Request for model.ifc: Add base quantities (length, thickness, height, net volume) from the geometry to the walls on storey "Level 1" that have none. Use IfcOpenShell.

First a look at what the model holds.

```python
import ifcopenshell
import ifcopenshell.util.element
import ifcopenshell.util.unit

model = ifcopenshell.open("model.ifc")
print(model.schema)
for unit_type in ("LENGTHUNIT", "AREAUNIT", "VOLUMEUNIT"):
    print(unit_type, ifcopenshell.util.unit.calculate_unit_scale(model, unit_type))
storey = next(s for s in model.by_type("IfcBuildingStorey") if s.Name == "Level 1")
walls = [e for e in ifcopenshell.util.element.get_decomposition(storey) if e.is_a("IfcWall")]
for e in sorted(walls, key=lambda e: e.id()):
    print(e.id(), e.is_a(), e.Name, list(ifcopenshell.util.element.get_psets(e, qtos_only=True)), sep=" | ")
```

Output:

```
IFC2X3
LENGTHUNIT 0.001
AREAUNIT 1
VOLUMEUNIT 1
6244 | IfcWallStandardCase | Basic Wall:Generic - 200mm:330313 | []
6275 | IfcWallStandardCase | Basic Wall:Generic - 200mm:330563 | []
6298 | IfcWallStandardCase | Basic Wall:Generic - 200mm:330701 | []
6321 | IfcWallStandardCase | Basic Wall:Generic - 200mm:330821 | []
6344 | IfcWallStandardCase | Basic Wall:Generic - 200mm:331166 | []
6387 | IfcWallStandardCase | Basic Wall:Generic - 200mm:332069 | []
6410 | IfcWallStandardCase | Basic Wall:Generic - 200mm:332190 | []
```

```python
import ifcopenshell
import ifcopenshell.api.pset
import ifcopenshell.geom
import ifcopenshell.util.element
import ifcopenshell.util.shape
import ifcopenshell.util.unit

model = ifcopenshell.open("model.ifc")
unit_scale = ifcopenshell.util.unit.calculate_unit_scale(model)
volume_scale = ifcopenshell.util.unit.calculate_unit_scale(model, "VOLUMEUNIT")
settings = ifcopenshell.geom.settings()

storey = next(s for s in model.by_type("IfcBuildingStorey") if s.Name == "Level 1")
walls = [e for e in ifcopenshell.util.element.get_decomposition(storey) if e.is_a("IfcWall")]

for e in sorted(walls, key=lambda e: e.id()):
    if ifcopenshell.util.element.get_psets(e, qtos_only=True, should_inherit=False):
        continue
    # Geometry comes back in metres, in the element's own axes.
    shape = ifcopenshell.geom.create_shape(settings, e)
    values = {
        "Length": ifcopenshell.util.shape.get_x(shape.geometry) / unit_scale,
        "Width": ifcopenshell.util.shape.get_y(shape.geometry) / unit_scale,
        "Height": ifcopenshell.util.shape.get_z(shape.geometry) / unit_scale,
        "NetVolume": ifcopenshell.util.shape.get_volume(shape.geometry) / volume_scale,
    }
    qto = ifcopenshell.api.pset.add_qto(model, product=e, name="BaseQuantities")
    ifcopenshell.api.pset.edit_qto(model, qto=qto, properties=values)
    print(e.id(), {k: round(v, 3) for k, v in values.items()})

model.write("model_v2.ifc")
```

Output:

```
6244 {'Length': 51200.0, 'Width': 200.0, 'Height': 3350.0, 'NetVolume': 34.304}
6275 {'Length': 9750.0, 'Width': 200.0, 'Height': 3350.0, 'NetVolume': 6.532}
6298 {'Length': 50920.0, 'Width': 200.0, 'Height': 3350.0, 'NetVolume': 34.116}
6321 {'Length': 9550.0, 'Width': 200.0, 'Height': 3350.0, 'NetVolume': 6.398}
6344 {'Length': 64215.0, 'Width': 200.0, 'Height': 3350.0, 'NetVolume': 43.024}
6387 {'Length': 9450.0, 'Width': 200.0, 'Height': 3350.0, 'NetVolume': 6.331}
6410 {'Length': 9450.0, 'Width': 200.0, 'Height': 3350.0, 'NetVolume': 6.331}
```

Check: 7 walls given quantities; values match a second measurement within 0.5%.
